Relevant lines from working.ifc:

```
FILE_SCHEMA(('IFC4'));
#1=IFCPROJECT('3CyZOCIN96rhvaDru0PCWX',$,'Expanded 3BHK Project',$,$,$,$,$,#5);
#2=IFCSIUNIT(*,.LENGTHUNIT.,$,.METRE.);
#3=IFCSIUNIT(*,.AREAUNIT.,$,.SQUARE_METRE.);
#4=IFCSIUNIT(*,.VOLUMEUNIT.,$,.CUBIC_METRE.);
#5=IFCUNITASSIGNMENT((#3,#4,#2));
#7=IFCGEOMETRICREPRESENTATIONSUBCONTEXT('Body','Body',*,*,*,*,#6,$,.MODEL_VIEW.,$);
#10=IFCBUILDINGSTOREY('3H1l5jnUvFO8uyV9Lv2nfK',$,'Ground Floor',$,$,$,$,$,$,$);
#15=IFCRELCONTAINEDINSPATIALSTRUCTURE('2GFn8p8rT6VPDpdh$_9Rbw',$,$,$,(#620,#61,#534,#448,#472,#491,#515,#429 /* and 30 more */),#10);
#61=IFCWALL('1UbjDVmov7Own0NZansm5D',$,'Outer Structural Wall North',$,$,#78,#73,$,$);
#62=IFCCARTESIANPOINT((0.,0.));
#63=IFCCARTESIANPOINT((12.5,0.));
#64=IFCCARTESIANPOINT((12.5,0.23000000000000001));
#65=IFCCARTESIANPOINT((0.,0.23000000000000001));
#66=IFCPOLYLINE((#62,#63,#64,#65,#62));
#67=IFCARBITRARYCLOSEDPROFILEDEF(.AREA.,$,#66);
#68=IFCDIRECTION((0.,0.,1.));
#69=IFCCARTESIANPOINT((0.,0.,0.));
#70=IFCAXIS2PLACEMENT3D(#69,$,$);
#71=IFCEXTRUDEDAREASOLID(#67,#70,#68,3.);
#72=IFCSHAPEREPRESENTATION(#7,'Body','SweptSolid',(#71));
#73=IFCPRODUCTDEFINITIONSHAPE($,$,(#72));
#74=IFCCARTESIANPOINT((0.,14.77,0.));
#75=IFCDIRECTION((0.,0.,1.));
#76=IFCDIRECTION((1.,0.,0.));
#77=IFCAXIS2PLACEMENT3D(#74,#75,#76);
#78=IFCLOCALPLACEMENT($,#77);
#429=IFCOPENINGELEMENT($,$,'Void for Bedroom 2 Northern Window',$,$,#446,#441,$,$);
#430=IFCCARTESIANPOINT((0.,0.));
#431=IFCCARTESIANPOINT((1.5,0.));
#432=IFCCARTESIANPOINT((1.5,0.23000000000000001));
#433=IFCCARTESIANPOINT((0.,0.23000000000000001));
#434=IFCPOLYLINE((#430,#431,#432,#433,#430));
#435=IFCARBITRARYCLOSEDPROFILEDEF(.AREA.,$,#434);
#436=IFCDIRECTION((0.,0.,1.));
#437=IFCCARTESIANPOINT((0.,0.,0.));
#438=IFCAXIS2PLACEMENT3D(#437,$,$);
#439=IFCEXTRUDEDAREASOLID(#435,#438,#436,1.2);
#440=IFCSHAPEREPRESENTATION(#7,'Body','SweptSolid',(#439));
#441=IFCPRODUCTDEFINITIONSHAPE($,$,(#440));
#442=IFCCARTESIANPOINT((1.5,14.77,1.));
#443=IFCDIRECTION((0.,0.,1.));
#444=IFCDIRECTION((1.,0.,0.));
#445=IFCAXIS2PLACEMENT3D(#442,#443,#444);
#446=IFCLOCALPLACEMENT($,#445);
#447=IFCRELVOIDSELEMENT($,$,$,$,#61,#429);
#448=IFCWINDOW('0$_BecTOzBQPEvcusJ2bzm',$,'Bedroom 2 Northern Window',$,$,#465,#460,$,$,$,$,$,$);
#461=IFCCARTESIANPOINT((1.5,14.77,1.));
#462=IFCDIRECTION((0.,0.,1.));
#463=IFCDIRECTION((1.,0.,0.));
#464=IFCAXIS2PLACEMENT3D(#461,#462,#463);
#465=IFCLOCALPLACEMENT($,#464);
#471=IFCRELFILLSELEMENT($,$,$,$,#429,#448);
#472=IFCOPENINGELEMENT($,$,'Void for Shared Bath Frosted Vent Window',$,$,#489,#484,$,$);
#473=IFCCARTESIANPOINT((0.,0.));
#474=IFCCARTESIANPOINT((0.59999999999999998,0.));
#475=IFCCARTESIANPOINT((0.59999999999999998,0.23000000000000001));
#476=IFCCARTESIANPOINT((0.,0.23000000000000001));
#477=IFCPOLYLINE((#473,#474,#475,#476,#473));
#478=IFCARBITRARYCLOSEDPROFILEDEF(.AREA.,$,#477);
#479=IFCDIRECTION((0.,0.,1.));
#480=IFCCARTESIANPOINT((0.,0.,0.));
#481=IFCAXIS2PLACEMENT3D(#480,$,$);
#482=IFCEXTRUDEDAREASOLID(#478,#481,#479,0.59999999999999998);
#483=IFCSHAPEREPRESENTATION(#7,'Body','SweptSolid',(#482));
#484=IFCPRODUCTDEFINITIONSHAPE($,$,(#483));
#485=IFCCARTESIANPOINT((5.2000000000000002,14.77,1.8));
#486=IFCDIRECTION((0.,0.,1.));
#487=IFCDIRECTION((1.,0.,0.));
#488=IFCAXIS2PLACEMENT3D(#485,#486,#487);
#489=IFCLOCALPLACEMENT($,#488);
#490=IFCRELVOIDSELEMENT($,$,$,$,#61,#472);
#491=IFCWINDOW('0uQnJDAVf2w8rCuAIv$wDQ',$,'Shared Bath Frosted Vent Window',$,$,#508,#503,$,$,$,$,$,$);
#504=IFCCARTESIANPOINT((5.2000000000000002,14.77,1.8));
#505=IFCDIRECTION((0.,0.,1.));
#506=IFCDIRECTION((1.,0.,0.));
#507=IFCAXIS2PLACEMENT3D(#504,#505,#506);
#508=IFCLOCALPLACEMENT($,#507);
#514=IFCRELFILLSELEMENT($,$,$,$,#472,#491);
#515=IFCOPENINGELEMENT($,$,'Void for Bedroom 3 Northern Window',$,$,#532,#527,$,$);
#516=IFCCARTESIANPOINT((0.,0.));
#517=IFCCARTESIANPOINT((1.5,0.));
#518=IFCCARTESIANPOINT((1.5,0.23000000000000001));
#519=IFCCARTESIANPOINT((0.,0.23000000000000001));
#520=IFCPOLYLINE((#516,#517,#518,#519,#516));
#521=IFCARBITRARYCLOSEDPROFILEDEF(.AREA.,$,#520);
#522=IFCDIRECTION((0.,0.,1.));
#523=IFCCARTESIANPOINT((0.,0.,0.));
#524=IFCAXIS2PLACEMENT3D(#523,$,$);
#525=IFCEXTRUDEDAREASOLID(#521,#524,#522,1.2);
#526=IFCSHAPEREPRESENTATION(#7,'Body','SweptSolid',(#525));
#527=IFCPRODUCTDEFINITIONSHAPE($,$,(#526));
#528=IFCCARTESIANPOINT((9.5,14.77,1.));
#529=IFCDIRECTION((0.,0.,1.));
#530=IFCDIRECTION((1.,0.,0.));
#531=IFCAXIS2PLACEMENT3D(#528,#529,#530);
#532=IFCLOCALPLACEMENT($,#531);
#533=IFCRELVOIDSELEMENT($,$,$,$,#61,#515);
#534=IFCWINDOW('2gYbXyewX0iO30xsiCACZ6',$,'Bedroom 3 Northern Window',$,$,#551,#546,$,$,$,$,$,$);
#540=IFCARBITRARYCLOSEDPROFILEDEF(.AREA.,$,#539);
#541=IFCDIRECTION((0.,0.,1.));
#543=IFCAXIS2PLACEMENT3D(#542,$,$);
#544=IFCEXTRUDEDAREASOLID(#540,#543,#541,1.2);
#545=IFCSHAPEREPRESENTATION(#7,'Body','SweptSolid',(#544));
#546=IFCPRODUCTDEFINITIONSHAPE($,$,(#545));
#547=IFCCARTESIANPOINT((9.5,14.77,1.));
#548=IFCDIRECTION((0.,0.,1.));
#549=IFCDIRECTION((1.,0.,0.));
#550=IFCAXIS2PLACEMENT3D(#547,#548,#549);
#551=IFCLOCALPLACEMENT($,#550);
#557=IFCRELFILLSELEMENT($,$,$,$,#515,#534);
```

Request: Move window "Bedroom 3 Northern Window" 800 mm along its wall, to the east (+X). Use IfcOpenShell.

```python
import ifcopenshell
import ifcopenshell.api.geometry
import ifcopenshell.util.placement

model = ifcopenshell.open("working.ifc")

window = model.by_guid("2gYbXyewX0iO30xsiCACZ6")
opening = window.FillsVoids[0].RelatingOpeningElement
wall = opening.VoidsElements[0].RelatingBuildingElement

wall_matrix = ifcopenshell.util.placement.get_local_placement(wall.ObjectPlacement)
shift = wall_matrix[:3, 0] * 0.8
before = ifcopenshell.util.placement.get_local_placement(window.ObjectPlacement)[:3, 3].copy()

# The window is not placed relative to its opening, so move both.
for product in (opening, window):
    matrix = ifcopenshell.util.placement.get_local_placement(product.ObjectPlacement)
    matrix[:3, 3] += shift
    ifcopenshell.api.geometry.edit_object_placement(model, product=product, matrix=matrix, is_si=False)

after = ifcopenshell.util.placement.get_local_placement(window.ObjectPlacement)[:3, 3]
print("window moved by", (after - before).round(3) + 0.0)

model.write("working_updated.ifc")
```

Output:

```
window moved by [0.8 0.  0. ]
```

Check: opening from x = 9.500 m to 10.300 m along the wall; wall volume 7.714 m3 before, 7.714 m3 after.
